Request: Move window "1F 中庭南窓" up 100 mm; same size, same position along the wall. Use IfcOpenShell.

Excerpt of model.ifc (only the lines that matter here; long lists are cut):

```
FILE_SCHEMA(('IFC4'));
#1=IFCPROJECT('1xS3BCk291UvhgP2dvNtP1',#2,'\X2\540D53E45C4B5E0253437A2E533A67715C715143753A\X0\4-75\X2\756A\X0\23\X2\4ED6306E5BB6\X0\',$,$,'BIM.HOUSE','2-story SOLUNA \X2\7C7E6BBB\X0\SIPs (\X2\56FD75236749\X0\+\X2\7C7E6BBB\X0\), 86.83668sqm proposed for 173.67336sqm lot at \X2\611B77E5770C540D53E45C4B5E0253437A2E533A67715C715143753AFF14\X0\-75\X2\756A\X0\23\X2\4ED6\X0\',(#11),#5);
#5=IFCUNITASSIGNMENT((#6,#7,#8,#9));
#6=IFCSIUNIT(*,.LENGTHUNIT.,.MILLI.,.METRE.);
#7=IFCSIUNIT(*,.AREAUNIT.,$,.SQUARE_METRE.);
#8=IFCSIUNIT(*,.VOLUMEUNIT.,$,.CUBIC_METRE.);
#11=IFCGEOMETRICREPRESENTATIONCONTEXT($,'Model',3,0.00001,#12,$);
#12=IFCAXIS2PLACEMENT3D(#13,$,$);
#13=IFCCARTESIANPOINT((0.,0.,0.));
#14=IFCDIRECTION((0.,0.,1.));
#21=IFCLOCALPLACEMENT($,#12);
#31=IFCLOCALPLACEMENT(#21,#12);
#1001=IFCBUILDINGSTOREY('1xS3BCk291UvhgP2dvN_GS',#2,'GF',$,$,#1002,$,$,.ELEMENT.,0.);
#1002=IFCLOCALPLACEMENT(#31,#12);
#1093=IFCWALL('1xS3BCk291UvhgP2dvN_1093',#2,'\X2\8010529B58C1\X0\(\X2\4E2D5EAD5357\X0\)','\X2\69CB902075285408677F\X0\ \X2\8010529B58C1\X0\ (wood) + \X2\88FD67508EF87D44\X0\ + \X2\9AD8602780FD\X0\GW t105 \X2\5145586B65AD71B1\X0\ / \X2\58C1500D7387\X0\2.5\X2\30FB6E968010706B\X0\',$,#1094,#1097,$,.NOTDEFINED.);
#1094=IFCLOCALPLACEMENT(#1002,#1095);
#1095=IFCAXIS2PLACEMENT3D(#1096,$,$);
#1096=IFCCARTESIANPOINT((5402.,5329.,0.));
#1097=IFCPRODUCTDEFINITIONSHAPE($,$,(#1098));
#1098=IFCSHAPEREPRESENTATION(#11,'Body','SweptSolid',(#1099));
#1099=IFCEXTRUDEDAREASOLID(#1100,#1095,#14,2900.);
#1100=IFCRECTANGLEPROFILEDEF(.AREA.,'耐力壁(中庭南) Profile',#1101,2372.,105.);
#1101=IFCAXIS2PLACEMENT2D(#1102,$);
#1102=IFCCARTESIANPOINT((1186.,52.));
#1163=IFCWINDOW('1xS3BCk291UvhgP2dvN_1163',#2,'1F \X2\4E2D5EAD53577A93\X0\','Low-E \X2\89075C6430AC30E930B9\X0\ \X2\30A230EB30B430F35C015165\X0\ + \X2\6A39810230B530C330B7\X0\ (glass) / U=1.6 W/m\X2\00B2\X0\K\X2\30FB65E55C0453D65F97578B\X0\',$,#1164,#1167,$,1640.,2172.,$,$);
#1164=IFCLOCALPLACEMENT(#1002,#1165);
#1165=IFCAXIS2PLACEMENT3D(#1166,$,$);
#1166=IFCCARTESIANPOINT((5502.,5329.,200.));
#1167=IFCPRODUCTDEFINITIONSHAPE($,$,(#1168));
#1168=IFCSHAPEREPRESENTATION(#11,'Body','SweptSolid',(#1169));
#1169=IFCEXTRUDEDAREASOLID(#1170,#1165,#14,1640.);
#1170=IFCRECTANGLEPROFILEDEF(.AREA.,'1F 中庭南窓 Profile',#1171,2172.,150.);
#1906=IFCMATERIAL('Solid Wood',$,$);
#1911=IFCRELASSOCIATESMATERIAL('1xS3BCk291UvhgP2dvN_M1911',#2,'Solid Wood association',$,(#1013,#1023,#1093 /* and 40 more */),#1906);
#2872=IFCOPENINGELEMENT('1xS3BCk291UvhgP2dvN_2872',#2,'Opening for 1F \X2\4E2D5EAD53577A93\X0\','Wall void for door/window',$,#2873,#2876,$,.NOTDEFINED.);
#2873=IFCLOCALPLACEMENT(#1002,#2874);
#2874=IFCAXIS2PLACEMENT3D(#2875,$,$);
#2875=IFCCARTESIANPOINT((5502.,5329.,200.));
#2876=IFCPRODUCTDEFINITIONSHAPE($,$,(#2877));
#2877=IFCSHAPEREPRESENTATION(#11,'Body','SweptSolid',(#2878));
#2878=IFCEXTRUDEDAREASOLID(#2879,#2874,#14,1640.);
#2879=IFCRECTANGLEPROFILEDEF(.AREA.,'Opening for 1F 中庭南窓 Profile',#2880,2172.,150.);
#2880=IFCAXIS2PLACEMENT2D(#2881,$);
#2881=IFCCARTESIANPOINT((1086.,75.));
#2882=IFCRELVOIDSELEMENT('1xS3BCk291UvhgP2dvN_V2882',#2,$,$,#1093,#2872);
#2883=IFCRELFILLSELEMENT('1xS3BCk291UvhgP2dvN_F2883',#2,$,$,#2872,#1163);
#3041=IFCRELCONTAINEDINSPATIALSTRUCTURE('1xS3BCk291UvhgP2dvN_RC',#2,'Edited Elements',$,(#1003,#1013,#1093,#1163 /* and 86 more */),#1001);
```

```python
import numpy as np
import ifcopenshell
import ifcopenshell.api.geometry
import ifcopenshell.util.placement
import ifcopenshell.util.unit

model = ifcopenshell.open("model.ifc")
unit_scale = ifcopenshell.util.unit.calculate_unit_scale(model)

window = model.by_guid("1xS3BCk291UvhgP2dvN_1163")
opening = window.FillsVoids[0].RelatingOpeningElement
dz = 100.0

shift = np.array([0.0, 0.0, dz])
# The window is not placed relative to its opening, so move both.
for product in (opening, window):
    matrix = ifcopenshell.util.placement.get_local_placement(product.ObjectPlacement)
    matrix[:3, 3] += shift
    ifcopenshell.api.geometry.edit_object_placement(model, product=product, matrix=matrix, is_si=False)

print(f"moved by {dz * unit_scale:+.3f} m")

model.write("model_rev.ifc")
```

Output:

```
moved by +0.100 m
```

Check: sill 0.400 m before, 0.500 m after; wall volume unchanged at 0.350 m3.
